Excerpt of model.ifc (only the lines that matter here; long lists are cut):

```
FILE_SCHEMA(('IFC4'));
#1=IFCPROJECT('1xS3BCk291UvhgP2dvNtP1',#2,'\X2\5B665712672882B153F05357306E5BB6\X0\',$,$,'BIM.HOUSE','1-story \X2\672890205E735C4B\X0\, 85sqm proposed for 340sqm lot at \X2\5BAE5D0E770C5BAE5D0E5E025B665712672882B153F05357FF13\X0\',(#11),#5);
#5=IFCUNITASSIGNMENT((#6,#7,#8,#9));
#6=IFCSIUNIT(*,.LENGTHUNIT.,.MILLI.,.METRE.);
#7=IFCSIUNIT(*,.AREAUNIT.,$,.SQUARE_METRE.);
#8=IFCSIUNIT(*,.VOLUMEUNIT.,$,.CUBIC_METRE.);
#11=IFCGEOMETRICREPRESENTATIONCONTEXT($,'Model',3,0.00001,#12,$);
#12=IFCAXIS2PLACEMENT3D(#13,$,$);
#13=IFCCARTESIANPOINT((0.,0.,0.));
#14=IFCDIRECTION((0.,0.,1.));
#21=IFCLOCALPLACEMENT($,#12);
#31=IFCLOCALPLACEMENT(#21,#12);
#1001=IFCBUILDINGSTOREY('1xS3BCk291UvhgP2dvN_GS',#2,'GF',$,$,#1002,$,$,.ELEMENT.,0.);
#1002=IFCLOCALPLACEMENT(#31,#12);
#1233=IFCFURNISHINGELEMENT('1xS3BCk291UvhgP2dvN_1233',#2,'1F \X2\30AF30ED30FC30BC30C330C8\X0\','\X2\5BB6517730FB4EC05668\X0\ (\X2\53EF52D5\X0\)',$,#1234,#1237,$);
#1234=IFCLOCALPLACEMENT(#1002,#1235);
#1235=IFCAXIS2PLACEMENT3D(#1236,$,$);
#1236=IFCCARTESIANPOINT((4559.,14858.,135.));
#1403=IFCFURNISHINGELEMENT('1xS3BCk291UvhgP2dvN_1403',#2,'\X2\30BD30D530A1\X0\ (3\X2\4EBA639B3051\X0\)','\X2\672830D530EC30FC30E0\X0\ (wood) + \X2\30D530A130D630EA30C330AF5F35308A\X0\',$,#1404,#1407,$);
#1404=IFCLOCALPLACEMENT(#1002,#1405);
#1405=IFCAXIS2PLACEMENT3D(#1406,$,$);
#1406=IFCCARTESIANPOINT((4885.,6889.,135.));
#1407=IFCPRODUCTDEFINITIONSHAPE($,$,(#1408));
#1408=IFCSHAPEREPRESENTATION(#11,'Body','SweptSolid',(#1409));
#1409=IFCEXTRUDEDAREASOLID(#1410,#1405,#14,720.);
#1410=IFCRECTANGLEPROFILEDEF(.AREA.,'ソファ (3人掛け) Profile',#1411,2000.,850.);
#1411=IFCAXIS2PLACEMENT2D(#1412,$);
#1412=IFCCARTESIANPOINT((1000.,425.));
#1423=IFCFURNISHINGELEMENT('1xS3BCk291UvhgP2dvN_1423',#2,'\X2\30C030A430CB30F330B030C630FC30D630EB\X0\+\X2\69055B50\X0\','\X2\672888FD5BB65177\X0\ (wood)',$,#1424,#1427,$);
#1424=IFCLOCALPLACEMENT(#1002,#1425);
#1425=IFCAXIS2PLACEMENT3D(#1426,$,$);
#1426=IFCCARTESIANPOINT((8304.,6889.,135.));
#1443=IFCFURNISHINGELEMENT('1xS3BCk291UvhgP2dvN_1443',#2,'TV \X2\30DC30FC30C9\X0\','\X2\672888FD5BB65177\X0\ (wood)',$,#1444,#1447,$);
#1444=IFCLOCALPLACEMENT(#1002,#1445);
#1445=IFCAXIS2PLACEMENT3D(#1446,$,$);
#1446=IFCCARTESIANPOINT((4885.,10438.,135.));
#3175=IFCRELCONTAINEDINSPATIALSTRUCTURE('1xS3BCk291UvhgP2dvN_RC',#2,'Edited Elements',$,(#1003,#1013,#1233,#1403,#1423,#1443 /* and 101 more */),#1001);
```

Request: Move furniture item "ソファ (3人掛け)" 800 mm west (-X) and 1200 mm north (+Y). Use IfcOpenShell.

```python
import ifcopenshell
import ifcopenshell.api.geometry
import ifcopenshell.util.placement

model = ifcopenshell.open("model.ifc")

item = model.by_id(1403)
matrix = ifcopenshell.util.placement.get_local_placement(item.ObjectPlacement)
matrix[0, 3] -= 800.0
matrix[1, 3] += 1200.0
ifcopenshell.api.geometry.edit_object_placement(model, product=item, matrix=matrix, is_si=False)

print(ifcopenshell.util.placement.get_local_placement(item.ObjectPlacement).round(3) + 0.0)

model.write("model_rev.ifc")
```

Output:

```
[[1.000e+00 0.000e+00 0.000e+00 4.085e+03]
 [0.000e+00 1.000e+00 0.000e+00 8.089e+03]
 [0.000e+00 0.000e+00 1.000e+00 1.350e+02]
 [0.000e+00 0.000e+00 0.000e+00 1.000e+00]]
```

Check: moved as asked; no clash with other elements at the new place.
